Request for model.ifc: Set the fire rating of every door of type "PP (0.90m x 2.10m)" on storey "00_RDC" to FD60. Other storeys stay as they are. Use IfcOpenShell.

First a look at what the model holds.

```python
import ifcopenshell
import ifcopenshell.util.element

model = ifcopenshell.open("model.ifc")
print(model.schema)
storey = next(s for s in model.by_type("IfcBuildingStorey") if s.Name == "00_RDC")
doors = [e for e in ifcopenshell.util.element.get_decomposition(storey) if e.is_a("IfcDoor")]
seen = {}
for e in doors:
    element_type = ifcopenshell.util.element.get_type(e)
    key = (element_type.Name if element_type != e and element_type else None, ifcopenshell.util.element.get_pset(e, "Pset_DoorCommon", "FireRating"))
    seen[key] = seen.get(key, 0) + 1
for (name, value), count in sorted(seen.items(), key=str):
    print(count, "x", name, "|", value)
```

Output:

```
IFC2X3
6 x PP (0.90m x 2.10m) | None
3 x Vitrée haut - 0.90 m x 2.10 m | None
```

```python
import ifcopenshell
import ifcopenshell.api.pset
import ifcopenshell.util.element

model = ifcopenshell.open("model.ifc")

storey = next(s for s in model.by_type("IfcBuildingStorey") if s.Name == "00_RDC")
doors = [e for e in ifcopenshell.util.element.get_decomposition(storey) if e.is_a("IfcDoor")]

count = 0
for e in doors:
    element_type = ifcopenshell.util.element.get_type(e)
    if element_type in (None, e) or element_type.Name != "PP (0.90m x 2.10m)":
        continue
    # add_pset returns the element's existing set when there is one.
    pset = ifcopenshell.api.pset.add_pset(model, product=e, name="Pset_DoorCommon")
    ifcopenshell.api.pset.edit_pset(model, pset=pset, properties={"FireRating": "FD60"})
    count += 1

print(count, "doors updated")

model.write("model_rev.ifc")
```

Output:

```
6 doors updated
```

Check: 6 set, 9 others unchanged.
